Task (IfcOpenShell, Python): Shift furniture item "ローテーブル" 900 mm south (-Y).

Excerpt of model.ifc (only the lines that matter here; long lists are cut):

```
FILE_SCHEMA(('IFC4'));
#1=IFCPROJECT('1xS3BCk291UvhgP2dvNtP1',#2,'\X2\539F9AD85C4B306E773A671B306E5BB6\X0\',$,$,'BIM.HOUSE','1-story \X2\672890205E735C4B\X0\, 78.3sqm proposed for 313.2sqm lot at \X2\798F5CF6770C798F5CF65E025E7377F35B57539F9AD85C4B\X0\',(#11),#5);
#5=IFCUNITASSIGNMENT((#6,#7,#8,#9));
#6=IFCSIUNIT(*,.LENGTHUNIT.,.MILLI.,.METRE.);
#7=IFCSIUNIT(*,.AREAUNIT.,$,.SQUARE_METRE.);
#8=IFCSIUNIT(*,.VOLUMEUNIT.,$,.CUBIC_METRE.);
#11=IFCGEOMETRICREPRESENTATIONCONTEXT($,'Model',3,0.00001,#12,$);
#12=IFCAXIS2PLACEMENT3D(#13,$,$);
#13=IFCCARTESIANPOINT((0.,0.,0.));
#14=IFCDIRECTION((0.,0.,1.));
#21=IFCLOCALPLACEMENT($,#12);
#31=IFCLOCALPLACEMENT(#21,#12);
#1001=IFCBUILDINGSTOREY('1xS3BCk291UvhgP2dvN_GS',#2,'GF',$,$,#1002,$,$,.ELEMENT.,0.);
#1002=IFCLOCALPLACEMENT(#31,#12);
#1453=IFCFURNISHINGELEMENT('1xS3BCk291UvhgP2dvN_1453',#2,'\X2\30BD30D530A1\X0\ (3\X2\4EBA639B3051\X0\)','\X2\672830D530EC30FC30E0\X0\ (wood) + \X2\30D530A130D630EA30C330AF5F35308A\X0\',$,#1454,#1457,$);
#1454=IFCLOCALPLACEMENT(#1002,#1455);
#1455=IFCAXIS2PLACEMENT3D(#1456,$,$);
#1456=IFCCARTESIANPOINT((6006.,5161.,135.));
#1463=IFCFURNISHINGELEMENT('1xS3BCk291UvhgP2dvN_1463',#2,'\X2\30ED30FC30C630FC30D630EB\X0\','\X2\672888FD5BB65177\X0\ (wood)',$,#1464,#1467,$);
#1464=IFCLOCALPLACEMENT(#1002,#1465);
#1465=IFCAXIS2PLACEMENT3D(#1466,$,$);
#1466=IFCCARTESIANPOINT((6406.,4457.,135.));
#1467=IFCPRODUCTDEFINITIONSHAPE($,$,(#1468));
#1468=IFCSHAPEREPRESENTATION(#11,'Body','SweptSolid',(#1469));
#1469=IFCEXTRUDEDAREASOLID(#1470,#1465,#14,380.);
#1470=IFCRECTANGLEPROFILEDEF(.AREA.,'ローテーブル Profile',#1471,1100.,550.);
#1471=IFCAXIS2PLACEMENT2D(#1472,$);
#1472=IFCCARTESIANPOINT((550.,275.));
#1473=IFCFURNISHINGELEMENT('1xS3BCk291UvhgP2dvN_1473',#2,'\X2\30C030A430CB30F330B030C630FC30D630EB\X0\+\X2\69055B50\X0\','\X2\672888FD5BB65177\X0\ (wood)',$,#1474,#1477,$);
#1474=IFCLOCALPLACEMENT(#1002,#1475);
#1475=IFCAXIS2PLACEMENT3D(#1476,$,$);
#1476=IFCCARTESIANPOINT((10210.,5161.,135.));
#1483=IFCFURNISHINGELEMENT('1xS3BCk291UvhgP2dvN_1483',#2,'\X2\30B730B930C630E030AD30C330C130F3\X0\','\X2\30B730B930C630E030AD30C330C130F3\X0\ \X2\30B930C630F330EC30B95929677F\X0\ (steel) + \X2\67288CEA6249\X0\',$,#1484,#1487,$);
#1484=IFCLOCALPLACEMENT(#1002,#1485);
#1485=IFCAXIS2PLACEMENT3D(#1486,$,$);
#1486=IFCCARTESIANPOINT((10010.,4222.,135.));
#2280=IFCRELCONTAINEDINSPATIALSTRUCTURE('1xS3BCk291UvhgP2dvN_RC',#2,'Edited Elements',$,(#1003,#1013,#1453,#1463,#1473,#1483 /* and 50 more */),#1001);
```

```python
import ifcopenshell
import ifcopenshell.api.geometry
import ifcopenshell.util.placement
import ifcopenshell.util.unit

model = ifcopenshell.open("model.ifc")
unit_scale = ifcopenshell.util.unit.calculate_unit_scale(model)

item = model.by_guid("1xS3BCk291UvhgP2dvN_1463")
matrix = ifcopenshell.util.placement.get_local_placement(item.ObjectPlacement)
matrix[1, 3] -= 0.9 / unit_scale
ifcopenshell.api.geometry.edit_object_placement(model, product=item, matrix=matrix, is_si=False)

print(ifcopenshell.util.placement.get_local_placement(item.ObjectPlacement).round(3) + 0.0)

model.write("model-out.ifc")
```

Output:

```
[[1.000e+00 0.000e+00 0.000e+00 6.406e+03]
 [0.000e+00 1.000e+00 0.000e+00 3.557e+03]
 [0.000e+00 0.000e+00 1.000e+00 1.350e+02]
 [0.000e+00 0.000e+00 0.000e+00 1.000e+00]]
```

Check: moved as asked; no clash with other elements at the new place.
